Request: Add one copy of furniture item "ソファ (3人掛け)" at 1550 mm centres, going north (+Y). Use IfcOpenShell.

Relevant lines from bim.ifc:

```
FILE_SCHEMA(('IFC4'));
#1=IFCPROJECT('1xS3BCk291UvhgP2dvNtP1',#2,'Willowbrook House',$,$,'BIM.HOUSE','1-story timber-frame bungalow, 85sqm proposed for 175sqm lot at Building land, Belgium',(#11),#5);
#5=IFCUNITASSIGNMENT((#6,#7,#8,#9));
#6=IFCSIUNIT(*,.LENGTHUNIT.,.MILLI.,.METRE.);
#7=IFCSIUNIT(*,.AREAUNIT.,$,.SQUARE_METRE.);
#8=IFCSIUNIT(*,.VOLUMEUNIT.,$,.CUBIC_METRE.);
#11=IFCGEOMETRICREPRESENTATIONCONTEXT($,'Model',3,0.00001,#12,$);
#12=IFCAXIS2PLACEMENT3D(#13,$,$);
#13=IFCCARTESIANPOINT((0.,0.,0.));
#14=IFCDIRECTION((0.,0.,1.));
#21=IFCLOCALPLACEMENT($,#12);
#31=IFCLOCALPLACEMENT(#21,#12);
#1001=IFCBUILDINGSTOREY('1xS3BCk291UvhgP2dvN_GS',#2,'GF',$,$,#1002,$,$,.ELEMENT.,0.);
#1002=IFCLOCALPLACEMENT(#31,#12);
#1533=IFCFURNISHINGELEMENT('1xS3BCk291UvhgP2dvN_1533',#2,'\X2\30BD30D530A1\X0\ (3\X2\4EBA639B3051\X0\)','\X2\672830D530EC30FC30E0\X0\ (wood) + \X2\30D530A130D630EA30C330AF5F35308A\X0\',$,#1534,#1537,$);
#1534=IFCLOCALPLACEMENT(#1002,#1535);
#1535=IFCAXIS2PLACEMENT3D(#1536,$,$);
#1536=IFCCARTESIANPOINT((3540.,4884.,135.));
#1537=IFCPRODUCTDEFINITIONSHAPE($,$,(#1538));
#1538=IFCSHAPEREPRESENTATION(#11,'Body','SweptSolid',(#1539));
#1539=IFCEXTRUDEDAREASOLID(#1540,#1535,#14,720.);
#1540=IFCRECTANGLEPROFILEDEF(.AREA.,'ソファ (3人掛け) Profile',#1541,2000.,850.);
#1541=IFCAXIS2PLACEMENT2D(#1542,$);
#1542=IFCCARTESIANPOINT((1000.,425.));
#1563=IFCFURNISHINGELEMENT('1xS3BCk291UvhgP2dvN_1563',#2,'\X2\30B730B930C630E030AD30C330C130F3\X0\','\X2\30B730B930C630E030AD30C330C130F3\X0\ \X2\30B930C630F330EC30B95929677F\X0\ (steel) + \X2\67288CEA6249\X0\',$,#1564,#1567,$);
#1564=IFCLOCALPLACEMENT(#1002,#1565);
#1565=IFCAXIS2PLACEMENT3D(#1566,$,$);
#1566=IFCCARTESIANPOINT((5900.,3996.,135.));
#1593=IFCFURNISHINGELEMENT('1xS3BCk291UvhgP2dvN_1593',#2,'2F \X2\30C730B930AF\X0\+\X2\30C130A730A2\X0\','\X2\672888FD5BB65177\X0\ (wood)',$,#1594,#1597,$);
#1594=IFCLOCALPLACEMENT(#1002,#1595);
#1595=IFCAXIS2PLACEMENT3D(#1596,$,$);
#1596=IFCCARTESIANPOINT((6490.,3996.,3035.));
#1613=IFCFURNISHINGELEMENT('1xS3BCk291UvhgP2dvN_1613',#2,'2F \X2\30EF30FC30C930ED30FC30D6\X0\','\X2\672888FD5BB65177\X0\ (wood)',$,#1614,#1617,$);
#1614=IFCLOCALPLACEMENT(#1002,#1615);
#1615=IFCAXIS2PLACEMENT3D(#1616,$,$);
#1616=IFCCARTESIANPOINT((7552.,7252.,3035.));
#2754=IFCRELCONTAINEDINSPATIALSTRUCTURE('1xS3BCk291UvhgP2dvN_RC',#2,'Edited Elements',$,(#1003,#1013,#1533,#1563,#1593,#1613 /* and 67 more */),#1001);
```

```python
import numpy as np
import ifcopenshell
import ifcopenshell.api.geometry
import ifcopenshell.api.root
import ifcopenshell.util.element
import ifcopenshell.util.placement

model = ifcopenshell.open("bim.ifc")


def reuse_history(source, copy):
    """copy_class also copies each property set's owner history, people and application; keep the originals."""
    for rel in copy.IsDefinedBy:
        if rel.is_a("IfcRelDefinesByProperties") and (history := rel.RelatingPropertyDefinition.OwnerHistory):
            rel.RelatingPropertyDefinition.OwnerHistory = source.OwnerHistory
            ifcopenshell.util.element.remove_deep2(model, history)


source = model.by_guid("1xS3BCk291UvhgP2dvN_1533")
base = ifcopenshell.util.placement.get_local_placement(source.ObjectPlacement)
step = np.array([0.0, 1.0, 0.0]) * 1550.0

for i in range(1, 2):
    copy = ifcopenshell.api.root.copy_class(model, product=source)
    copy.Representation = ifcopenshell.util.element.copy_deep(
        model, source.Representation, exclude=["IfcGeometricRepresentationContext", "IfcRepresentationMap"]
    )
    reuse_history(source, copy)
    matrix = base.copy()
    matrix[:3, 3] += i * step
    print("added at", matrix[:3, 3].round(3) + 0.0)
    ifcopenshell.api.geometry.edit_object_placement(model, product=copy, matrix=matrix, is_si=False)

model.write("bim_edited.ifc")
```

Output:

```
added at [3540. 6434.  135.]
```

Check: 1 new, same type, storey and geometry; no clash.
